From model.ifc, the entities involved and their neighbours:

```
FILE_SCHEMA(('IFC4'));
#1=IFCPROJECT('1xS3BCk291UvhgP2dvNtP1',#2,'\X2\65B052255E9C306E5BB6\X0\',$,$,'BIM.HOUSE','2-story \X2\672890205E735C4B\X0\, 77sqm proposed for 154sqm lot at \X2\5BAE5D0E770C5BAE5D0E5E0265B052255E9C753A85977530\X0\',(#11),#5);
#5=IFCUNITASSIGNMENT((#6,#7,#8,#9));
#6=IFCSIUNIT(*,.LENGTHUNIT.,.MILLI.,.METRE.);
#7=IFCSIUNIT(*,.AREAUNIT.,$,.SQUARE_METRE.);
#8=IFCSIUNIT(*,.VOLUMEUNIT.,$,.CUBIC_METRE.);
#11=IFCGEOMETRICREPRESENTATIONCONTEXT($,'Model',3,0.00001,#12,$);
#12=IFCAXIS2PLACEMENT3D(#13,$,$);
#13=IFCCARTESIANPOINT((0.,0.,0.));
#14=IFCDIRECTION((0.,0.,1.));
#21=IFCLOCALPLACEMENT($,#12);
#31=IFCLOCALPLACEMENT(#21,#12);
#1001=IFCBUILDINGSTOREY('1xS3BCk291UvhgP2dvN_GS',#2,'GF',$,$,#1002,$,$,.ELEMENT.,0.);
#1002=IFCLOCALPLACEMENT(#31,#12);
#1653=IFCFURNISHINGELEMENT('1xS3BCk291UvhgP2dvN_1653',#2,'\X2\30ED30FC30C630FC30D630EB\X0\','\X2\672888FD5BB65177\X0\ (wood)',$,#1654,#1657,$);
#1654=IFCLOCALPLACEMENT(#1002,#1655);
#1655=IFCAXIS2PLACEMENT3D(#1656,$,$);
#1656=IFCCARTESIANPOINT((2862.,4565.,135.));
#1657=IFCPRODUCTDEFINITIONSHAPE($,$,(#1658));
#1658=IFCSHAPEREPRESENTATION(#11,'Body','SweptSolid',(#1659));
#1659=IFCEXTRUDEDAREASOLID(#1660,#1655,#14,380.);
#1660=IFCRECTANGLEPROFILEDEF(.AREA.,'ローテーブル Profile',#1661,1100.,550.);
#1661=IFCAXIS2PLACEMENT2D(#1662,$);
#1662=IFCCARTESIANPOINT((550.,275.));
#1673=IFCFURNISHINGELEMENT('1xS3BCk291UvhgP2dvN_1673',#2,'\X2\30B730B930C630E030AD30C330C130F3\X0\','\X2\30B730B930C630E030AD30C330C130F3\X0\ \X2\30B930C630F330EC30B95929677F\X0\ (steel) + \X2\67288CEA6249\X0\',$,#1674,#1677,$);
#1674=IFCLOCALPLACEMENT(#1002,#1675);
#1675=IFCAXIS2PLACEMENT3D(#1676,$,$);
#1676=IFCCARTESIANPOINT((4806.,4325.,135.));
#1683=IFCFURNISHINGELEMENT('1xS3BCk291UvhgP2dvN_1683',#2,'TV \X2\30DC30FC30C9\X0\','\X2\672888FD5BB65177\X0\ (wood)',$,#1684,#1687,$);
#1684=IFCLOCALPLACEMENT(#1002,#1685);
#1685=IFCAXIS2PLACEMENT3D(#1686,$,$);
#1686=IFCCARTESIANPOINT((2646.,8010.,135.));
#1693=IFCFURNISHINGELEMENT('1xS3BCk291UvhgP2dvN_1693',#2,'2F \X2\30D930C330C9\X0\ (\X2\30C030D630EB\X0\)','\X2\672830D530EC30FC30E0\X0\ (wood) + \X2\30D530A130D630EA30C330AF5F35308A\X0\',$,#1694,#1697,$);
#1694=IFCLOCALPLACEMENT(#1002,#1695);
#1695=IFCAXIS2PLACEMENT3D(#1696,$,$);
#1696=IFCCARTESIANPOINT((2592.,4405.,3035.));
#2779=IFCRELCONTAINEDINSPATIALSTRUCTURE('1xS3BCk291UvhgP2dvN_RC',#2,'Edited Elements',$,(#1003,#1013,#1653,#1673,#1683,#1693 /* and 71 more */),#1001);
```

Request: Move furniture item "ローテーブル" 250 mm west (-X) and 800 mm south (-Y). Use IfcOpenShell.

```python
import ifcopenshell
import ifcopenshell.api.geometry
import ifcopenshell.util.placement

model = ifcopenshell.open("model.ifc")

item = model.by_guid("1xS3BCk291UvhgP2dvN_1653")
matrix = ifcopenshell.util.placement.get_local_placement(item.ObjectPlacement)
matrix[0, 3] -= 250.0
matrix[1, 3] -= 800.0
ifcopenshell.api.geometry.edit_object_placement(model, product=item, matrix=matrix, is_si=False)

print(ifcopenshell.util.placement.get_local_placement(item.ObjectPlacement).round(3) + 0.0)

model.write("model_edited.ifc")
```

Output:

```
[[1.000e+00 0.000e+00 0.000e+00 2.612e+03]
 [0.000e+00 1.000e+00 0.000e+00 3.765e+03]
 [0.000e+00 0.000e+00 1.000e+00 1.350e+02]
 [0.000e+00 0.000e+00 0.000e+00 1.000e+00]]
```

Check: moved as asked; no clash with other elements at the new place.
